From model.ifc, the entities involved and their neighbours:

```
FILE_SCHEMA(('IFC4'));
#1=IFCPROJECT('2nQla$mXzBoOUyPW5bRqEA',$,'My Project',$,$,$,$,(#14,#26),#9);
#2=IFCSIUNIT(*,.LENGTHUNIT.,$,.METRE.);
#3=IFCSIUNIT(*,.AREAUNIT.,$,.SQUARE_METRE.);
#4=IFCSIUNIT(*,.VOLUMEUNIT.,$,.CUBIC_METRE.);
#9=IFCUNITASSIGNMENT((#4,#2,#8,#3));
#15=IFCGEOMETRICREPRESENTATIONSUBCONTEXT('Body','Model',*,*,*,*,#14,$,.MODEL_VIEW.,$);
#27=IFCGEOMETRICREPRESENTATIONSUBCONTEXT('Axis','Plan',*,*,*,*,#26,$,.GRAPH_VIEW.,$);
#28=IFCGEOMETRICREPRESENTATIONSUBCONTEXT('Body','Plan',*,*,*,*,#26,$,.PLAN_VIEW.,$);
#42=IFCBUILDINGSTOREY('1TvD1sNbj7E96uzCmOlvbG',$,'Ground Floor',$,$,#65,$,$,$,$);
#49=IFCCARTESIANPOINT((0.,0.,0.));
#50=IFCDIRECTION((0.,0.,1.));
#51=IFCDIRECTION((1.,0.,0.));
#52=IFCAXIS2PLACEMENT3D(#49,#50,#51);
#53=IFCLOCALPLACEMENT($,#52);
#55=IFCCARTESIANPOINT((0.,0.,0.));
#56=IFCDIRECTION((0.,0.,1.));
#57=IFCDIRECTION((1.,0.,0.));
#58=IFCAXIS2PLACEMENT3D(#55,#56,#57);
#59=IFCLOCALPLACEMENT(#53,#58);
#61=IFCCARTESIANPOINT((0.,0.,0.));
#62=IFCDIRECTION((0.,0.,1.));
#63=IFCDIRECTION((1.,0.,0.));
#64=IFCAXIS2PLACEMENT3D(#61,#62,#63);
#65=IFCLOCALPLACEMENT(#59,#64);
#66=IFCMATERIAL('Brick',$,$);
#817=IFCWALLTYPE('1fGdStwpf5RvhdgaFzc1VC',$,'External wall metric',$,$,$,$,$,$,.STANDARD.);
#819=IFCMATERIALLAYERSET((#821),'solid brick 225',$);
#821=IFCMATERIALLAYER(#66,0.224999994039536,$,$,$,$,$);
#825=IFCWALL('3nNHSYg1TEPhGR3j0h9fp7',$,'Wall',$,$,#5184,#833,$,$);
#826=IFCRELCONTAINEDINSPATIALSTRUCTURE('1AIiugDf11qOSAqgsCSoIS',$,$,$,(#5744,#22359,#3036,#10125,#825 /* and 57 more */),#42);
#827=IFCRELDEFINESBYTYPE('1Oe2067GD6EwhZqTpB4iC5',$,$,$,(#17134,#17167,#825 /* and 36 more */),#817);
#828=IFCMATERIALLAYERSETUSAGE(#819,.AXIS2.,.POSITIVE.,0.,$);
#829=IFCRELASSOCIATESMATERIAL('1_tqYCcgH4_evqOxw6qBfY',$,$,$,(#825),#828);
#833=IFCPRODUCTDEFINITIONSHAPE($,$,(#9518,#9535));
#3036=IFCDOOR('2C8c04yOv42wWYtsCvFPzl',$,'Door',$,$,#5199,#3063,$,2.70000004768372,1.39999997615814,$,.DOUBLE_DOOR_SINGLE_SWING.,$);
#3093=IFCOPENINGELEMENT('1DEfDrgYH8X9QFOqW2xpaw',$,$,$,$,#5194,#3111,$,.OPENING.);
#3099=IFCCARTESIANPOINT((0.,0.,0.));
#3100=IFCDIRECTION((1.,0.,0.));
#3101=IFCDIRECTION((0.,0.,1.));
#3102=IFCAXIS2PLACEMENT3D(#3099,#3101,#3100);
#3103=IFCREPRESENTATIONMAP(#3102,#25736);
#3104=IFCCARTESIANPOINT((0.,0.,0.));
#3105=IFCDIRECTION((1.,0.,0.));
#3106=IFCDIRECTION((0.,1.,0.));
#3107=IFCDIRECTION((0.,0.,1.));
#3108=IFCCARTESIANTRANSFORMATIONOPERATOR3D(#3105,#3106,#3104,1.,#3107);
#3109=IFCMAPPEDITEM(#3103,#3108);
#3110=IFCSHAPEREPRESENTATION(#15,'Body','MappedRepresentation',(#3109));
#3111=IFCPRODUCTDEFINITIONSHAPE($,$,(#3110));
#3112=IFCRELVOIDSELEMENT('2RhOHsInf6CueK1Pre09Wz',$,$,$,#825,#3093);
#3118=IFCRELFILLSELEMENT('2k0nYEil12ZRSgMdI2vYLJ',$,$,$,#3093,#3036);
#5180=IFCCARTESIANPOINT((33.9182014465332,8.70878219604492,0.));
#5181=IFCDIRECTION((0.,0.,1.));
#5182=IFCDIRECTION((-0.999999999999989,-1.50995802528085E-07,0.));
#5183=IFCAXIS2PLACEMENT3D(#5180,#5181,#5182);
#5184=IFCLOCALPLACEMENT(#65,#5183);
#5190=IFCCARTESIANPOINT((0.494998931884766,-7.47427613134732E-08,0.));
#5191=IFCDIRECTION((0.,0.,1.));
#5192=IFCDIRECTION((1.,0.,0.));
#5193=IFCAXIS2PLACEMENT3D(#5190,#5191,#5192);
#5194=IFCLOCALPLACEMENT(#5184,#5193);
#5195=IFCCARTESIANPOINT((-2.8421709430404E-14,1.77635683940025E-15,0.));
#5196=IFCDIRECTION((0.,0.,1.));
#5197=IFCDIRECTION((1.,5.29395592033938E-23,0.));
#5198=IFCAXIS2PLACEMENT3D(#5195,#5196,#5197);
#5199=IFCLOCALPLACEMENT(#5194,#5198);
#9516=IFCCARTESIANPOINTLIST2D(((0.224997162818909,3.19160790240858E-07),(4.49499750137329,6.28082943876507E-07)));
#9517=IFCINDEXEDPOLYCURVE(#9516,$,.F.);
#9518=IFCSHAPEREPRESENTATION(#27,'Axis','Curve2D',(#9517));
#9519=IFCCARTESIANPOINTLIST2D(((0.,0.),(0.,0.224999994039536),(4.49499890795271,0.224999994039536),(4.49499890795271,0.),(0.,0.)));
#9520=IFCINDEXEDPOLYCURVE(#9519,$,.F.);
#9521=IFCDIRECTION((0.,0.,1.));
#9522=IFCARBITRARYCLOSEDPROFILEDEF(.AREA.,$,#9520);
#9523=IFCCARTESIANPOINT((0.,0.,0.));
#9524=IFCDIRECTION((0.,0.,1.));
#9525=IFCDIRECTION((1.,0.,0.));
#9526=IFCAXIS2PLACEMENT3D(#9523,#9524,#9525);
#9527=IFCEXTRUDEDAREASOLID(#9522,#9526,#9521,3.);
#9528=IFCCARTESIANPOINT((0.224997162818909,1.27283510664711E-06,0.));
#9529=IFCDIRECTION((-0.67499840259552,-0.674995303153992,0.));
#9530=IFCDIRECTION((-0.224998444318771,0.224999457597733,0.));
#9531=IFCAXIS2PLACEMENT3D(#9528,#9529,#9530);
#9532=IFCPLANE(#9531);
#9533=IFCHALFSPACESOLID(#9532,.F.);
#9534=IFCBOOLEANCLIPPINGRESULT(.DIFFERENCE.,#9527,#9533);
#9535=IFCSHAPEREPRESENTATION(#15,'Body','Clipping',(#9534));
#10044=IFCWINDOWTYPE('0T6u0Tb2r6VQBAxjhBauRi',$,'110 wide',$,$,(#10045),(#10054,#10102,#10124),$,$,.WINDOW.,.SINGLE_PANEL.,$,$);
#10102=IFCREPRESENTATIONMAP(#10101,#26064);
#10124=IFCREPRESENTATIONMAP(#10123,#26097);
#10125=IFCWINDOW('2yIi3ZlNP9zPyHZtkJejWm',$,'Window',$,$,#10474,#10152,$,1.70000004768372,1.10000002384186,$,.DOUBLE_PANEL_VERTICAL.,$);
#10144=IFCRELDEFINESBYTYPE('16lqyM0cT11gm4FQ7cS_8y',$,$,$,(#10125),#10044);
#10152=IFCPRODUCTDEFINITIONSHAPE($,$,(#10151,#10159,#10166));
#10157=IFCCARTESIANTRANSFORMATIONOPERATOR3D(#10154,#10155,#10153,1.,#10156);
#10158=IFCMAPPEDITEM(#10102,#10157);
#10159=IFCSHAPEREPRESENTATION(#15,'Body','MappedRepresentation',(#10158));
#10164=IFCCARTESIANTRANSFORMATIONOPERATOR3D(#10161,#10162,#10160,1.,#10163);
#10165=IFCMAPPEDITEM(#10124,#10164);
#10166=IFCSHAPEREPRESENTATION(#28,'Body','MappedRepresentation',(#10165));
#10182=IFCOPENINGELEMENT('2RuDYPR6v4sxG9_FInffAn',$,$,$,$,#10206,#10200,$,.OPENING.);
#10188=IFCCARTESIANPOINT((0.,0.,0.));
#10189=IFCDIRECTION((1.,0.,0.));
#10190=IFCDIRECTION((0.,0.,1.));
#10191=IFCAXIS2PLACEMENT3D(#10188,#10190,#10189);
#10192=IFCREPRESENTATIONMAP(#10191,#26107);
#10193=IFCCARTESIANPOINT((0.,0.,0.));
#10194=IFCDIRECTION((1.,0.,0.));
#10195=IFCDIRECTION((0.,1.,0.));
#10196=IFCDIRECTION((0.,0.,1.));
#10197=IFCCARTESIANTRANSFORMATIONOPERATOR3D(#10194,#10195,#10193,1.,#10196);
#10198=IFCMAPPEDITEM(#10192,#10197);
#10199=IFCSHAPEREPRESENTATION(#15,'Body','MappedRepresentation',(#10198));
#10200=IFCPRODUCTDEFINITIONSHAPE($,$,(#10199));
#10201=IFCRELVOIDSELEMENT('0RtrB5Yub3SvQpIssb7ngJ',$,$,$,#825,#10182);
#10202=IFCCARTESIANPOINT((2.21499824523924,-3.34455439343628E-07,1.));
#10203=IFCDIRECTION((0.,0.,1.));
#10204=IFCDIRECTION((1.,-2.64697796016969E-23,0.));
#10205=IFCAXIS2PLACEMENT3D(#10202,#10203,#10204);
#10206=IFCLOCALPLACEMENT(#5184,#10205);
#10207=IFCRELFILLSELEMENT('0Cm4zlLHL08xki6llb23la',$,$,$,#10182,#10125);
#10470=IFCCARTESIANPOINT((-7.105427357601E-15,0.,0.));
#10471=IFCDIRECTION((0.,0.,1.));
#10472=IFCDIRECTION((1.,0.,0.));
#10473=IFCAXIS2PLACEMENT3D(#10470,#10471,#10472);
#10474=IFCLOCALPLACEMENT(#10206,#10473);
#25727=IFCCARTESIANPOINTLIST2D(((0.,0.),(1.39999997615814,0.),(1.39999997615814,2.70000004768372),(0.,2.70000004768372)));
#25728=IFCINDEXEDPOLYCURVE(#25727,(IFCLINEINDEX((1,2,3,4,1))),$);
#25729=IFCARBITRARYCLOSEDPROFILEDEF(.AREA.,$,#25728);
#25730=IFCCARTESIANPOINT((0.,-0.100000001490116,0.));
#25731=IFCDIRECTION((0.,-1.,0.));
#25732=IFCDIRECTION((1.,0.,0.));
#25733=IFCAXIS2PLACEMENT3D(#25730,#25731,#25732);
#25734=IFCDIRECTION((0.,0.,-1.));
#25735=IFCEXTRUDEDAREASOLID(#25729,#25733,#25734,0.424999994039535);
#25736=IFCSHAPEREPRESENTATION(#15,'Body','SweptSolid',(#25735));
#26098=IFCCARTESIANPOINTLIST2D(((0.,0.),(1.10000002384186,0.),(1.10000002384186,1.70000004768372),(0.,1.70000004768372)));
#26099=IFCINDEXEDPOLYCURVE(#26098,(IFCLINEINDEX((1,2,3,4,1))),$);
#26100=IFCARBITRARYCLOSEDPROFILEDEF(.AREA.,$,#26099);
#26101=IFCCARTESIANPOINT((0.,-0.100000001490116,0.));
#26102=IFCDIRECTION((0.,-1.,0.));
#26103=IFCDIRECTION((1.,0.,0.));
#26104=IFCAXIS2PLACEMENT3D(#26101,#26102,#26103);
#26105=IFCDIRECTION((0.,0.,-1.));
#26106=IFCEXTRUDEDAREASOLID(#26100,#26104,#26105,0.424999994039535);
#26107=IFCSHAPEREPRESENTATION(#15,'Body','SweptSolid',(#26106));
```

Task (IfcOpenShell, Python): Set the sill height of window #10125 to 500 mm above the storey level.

```python
import numpy as np
import ifcopenshell
import ifcopenshell.api.geometry
import ifcopenshell.geom
import ifcopenshell.util.element
import ifcopenshell.util.placement
import ifcopenshell.util.shape
import ifcopenshell.util.unit

model = ifcopenshell.open("model.ifc")
unit_scale = ifcopenshell.util.unit.calculate_unit_scale(model)

window = model.by_id(10125)
opening = window.FillsVoids[0].RelatingOpeningElement
storey = ifcopenshell.util.element.get_container(window, ifc_class="IfcBuildingStorey")
level = ifcopenshell.util.placement.get_local_placement(storey.ObjectPlacement)[2, 3]

# The opening's origin need not be at the sill, so measure its lowest point.
shape = ifcopenshell.geom.create_shape(ifcopenshell.geom.settings(), opening)
bottom = ifcopenshell.util.shape.get_shape_bottom_elevation(shape, shape.geometry) / unit_scale
dz = level + 0.5 - bottom

shift = np.array([0.0, 0.0, dz])
# The window is placed relative to its opening, so it follows when the opening moves.
matrix = ifcopenshell.util.placement.get_local_placement(opening.ObjectPlacement)
matrix[:3, 3] += shift
ifcopenshell.api.geometry.edit_object_placement(
    model, product=opening, matrix=matrix, is_si=False, should_transform_children=True
)

print(f"moved by {dz * unit_scale:+.3f} m")

model.write("model_edited.ifc")
```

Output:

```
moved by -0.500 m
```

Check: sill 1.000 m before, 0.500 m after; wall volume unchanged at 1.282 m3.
